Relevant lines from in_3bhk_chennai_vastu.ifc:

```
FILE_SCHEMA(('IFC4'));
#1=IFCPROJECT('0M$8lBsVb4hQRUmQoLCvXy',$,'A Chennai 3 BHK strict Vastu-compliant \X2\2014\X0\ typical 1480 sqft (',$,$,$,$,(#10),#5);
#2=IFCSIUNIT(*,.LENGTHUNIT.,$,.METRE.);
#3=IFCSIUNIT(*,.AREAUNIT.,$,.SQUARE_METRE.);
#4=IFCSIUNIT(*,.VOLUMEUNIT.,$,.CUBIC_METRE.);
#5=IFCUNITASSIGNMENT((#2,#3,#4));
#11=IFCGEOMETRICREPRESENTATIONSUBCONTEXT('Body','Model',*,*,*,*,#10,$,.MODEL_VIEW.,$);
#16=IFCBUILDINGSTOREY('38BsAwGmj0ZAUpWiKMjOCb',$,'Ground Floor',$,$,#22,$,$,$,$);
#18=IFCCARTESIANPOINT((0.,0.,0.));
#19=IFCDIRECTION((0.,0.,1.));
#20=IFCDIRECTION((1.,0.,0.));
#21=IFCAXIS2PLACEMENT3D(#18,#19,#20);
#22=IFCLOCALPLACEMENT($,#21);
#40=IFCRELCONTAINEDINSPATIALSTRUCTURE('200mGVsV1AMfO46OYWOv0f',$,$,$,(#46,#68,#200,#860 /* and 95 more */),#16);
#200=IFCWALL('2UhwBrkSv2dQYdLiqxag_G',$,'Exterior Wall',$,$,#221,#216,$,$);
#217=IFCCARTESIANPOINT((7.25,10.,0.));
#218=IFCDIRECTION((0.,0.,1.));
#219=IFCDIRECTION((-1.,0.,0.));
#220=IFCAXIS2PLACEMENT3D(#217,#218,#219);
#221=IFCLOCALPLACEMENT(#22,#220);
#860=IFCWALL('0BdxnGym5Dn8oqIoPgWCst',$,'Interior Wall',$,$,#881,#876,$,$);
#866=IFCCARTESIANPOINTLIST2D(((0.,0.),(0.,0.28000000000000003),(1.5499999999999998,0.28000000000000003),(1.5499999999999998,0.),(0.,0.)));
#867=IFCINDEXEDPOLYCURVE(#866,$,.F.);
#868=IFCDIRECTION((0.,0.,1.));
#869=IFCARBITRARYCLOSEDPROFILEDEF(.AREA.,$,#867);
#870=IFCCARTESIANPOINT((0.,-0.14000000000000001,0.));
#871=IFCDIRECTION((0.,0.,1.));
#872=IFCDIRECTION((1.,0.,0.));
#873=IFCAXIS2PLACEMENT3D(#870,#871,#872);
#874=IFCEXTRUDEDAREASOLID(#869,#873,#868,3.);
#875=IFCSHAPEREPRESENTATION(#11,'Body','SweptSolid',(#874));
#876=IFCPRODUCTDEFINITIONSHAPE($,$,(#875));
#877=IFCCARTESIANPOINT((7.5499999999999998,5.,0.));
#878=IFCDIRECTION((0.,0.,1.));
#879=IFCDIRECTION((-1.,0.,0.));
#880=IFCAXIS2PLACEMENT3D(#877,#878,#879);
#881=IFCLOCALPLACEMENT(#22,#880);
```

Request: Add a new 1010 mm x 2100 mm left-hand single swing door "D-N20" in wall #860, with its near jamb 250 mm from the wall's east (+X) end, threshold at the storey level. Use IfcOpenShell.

```python
import numpy as np
import ifcopenshell
import ifcopenshell.api.feature
import ifcopenshell.api.geometry
import ifcopenshell.api.root
import ifcopenshell.api.spatial
import ifcopenshell.geom
import ifcopenshell.util.element
import ifcopenshell.util.placement
import ifcopenshell.util.representation
import ifcopenshell.util.shape
import ifcopenshell.util.unit

model = ifcopenshell.open("in_3bhk_chennai_vastu.ifc")
unit_scale = ifcopenshell.util.unit.calculate_unit_scale(model)
settings = ifcopenshell.geom.settings()


def volume(element):
    """Net volume in cubic metres, openings subtracted."""
    shape = ifcopenshell.geom.create_shape(settings, element)
    return ifcopenshell.util.shape.get_volume(shape.geometry)


wall = model.by_guid("0BdxnGym5Dn8oqIoPgWCst")
storey = ifcopenshell.util.element.get_container(wall, ifc_class="IfcBuildingStorey")
context = ifcopenshell.util.representation.get_context(model, "Model", "Body", "MODEL_VIEW")
before = volume(wall)

width, height, from_end, sill = 1.01, 2.1, 0.25, 0.0  # metres

# The wall runs along its own X axis, and the end named is its -X end.
wall_shape = ifcopenshell.geom.create_shape(settings, wall)
x, y, z = ifcopenshell.util.shape.get_vertices(wall_shape.geometry).T
start = x.min() + from_end
face, thickness = float(y.min()), float(y.max() - y.min())
wall_matrix = ifcopenshell.util.placement.get_local_placement(wall.ObjectPlacement)
level = ifcopenshell.util.placement.get_local_placement(storey.ObjectPlacement)[2, 3]


def in_wall(x, y):
    """Placement at x, y metres in the wall's axes, at sill height."""
    matrix = wall_matrix.copy()
    matrix[:, 3] = wall_matrix @ np.array([x / unit_scale, y / unit_scale, 0.0, 1.0])
    matrix[2, 3] = level + sill / unit_scale
    return matrix


# Opening: a box that overshoots both wall faces by 50 mm.
opening = ifcopenshell.api.root.create_entity(model, ifc_class="IfcOpeningElement", predefined_type="OPENING")
box = ifcopenshell.api.geometry.add_wall_representation(
    model, context=context, length=width, height=height, thickness=thickness + 0.1
)
ifcopenshell.api.geometry.assign_representation(model, product=opening, representation=box)
ifcopenshell.api.geometry.edit_object_placement(model, product=opening, matrix=in_wall(start, face - 0.05), is_si=False)
ifcopenshell.api.feature.add_feature(model, feature=opening, element=wall)

door = ifcopenshell.api.root.create_entity(model, ifc_class="IfcDoor", name="D-N20", predefined_type="DOOR")
door.OverallWidth, door.OverallHeight = width / unit_scale, height / unit_scale
door.OperationType = "SINGLE_SWING_LEFT"
body = ifcopenshell.api.geometry.add_door_representation(
    model,
    context=context,
    overall_width=door.OverallWidth,
    overall_height=door.OverallHeight,
    operation_type="SINGLE_SWING_LEFT",
    lining_properties={"LiningDepth": thickness / unit_scale, "ThresholdDepth": thickness / unit_scale},
)
ifcopenshell.api.geometry.assign_representation(model, product=door, representation=body)
ifcopenshell.api.spatial.assign_container(model, products=[door], relating_structure=storey)
ifcopenshell.api.feature.add_filling(model, opening=opening, element=door)

# The lining spans the wall, so the door starts at the wall face.
ifcopenshell.api.geometry.edit_object_placement(model, product=door, matrix=in_wall(start, face), is_si=False)

after = volume(wall)

print(f"wall volume {before:.3f} -> {after:.3f} m3")

model.write("in_3bhk_chennai_vastu_rev.ifc")
```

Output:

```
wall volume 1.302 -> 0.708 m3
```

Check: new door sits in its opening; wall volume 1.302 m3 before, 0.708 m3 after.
